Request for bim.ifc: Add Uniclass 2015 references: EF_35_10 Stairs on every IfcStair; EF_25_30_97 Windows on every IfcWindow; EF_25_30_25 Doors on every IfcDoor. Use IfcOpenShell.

First a look at what the model holds.

```python
import ifcopenshell

model = ifcopenshell.open("bim.ifc")
print(model.schema)
print("classifications:", [c.Name for c in model.by_type("IfcClassification")])
for ifc_class in ("IfcDoor", "IfcRoof", "IfcStair", "IfcWall", "IfcWindow"):
    print(ifc_class, len(model.by_type(ifc_class)))
```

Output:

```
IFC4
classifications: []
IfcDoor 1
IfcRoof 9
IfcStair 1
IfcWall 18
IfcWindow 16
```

```python
import ifcopenshell
import ifcopenshell.api.classification

model = ifcopenshell.open("bim.ifc")

system = ifcopenshell.api.classification.add_classification(model, classification="Uniclass 2015")

codes = {
    "IfcStair": ("EF_35_10", "Stairs"),
    "IfcWindow": ("EF_25_30_97", "Windows"),
    "IfcDoor": ("EF_25_30_25", "Doors"),
}
for ifc_class, (code, name) in codes.items():
    products = model.by_type(ifc_class)
    ifcopenshell.api.classification.add_reference(
        model, products=products, classification=system, identification=code, name=name
    )
    print(code, len(products))

model.write("bim_updated.ifc")
```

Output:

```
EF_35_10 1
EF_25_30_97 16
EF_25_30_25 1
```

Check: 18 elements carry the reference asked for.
